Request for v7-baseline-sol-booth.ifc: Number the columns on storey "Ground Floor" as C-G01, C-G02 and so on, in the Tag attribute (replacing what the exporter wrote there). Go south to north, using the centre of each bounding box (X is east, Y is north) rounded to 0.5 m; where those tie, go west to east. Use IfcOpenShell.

First a look at what the model holds.

```python
import ifcopenshell
import ifcopenshell.util.element
import ifcopenshell.util.placement

model = ifcopenshell.open("v7-baseline-sol-booth.ifc")
print(model.schema)
storey = next(s for s in model.by_type("IfcBuildingStorey") if s.Name == "Ground Floor")
columns = [e for e in ifcopenshell.util.element.get_decomposition(storey) if e.is_a("IfcColumn")]
for e in sorted(columns, key=lambda e: e.id()):
    origin = ifcopenshell.util.placement.get_local_placement(e.ObjectPlacement)[:3, 3]
    print(e.id(), e.Tag, e.Name, origin.round(2) + 0.0, sep=" | ")
```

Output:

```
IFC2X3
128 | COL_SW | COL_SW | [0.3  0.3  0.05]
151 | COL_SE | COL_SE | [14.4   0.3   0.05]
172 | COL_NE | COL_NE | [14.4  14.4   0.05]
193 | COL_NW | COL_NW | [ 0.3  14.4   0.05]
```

```python
import ifcopenshell
import ifcopenshell.geom
import ifcopenshell.util.element
import ifcopenshell.util.shape

model = ifcopenshell.open("v7-baseline-sol-booth.ifc")
settings = ifcopenshell.geom.settings()
settings.set("use-world-coords", True)


def centre(element):
    shape = ifcopenshell.geom.create_shape(settings, element)
    return ifcopenshell.util.shape.get_bbox_centroid(shape.geometry)


storey = next(s for s in model.by_type("IfcBuildingStorey") if s.Name == "Ground Floor")
columns = [e for e in ifcopenshell.util.element.get_decomposition(storey) if e.is_a("IfcColumn")]

# Insertion points can sit at a corner or the storey origin, so sort by the geometry (in metres).
centres = {e: centre(e) for e in columns}
columns.sort(key=lambda e: (round(centres[e][1] / 0.5), centres[e][0]))

for i, e in enumerate(columns, start=1):
    number = f"C-G{i:02d}"
    e.Tag = number
    print(e.id(), number)

model.write("v7-baseline-sol-booth-out.ifc")
```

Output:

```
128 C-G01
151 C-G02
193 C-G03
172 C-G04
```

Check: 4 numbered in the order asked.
